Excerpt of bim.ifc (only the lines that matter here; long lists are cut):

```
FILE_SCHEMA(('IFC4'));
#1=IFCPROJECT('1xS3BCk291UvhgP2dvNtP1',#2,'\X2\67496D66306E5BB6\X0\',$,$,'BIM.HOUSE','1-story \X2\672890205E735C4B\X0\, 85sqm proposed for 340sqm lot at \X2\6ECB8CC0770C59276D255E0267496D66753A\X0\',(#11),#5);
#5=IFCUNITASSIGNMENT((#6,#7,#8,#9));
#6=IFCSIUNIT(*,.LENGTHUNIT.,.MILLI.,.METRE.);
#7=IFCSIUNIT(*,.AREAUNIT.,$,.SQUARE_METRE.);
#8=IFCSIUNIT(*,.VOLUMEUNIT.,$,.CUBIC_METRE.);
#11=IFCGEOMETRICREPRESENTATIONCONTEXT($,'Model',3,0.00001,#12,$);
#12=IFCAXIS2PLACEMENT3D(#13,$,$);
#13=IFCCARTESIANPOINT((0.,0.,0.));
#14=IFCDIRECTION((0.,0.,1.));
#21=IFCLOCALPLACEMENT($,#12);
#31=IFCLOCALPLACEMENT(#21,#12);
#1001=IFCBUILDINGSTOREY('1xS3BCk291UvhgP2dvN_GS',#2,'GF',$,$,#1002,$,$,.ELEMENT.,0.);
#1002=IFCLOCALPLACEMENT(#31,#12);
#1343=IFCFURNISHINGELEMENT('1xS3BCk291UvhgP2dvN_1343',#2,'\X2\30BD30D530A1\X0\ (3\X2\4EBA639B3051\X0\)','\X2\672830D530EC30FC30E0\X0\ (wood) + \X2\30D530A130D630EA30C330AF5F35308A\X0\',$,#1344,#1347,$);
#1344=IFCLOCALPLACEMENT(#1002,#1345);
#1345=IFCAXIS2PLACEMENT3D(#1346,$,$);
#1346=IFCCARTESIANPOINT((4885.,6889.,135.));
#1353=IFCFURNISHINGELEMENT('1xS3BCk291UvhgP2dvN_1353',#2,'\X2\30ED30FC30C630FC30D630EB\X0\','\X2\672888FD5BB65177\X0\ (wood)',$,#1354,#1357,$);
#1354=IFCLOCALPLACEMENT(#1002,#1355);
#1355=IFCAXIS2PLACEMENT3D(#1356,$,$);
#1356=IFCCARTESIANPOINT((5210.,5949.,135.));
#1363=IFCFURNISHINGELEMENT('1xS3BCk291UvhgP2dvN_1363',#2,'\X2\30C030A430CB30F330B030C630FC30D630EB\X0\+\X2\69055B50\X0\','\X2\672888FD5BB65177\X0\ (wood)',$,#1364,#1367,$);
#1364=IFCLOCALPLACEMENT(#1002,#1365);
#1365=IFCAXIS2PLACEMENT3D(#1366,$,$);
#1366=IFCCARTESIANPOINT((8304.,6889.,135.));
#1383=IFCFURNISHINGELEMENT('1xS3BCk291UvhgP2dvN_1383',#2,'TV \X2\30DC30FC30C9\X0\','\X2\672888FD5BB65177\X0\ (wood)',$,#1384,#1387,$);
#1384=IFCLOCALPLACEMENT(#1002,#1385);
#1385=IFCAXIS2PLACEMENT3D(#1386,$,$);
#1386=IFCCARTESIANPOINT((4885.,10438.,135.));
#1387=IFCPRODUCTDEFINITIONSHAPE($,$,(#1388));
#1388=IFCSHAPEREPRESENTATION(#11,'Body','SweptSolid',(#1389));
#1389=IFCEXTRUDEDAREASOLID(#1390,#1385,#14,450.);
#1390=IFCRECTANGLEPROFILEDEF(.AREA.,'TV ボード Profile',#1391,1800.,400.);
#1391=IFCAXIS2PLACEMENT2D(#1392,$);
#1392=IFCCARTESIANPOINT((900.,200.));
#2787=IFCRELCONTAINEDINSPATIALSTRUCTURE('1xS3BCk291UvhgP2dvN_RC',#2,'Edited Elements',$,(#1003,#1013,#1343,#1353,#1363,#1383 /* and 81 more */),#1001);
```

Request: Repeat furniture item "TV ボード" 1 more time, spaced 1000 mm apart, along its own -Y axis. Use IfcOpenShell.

```python
import ifcopenshell
import ifcopenshell.api.geometry
import ifcopenshell.api.root
import ifcopenshell.util.element
import ifcopenshell.util.placement
import ifcopenshell.util.unit

model = ifcopenshell.open("bim.ifc")
unit_scale = ifcopenshell.util.unit.calculate_unit_scale(model)


def reuse_history(source, copy):
    """copy_class also copies each property set's owner history, people and application; keep the originals."""
    for rel in copy.IsDefinedBy:
        if rel.is_a("IfcRelDefinesByProperties") and (history := rel.RelatingPropertyDefinition.OwnerHistory):
            rel.RelatingPropertyDefinition.OwnerHistory = source.OwnerHistory
            ifcopenshell.util.element.remove_deep2(model, history)


source = model.by_id(1383)
base = ifcopenshell.util.placement.get_local_placement(source.ObjectPlacement)
step = -base[:3, 1] * 1 / unit_scale

for i in range(1, 2):
    copy = ifcopenshell.api.root.copy_class(model, product=source)
    copy.Representation = ifcopenshell.util.element.copy_deep(
        model, source.Representation, exclude=["IfcGeometricRepresentationContext", "IfcRepresentationMap"]
    )
    reuse_history(source, copy)
    matrix = base.copy()
    matrix[:3, 3] += i * step
    print("added at", matrix[:3, 3].round(3) + 0.0)
    ifcopenshell.api.geometry.edit_object_placement(model, product=copy, matrix=matrix, is_si=False)

model.write("bim_edited.ifc")
```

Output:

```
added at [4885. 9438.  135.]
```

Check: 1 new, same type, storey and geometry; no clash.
